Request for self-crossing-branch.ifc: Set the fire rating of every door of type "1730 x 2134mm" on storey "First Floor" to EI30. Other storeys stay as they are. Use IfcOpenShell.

First a look at what the model holds.

```python
import ifcopenshell
import ifcopenshell.util.element

model = ifcopenshell.open("self-crossing-branch.ifc")
print(model.schema)
storey = next(s for s in model.by_type("IfcBuildingStorey") if s.Name == "First Floor")
doors = [e for e in ifcopenshell.util.element.get_decomposition(storey) if e.is_a("IfcDoor")]
seen = {}
for e in doors:
    element_type = ifcopenshell.util.element.get_type(e)
    key = (element_type.Name if element_type != e and element_type else None, ifcopenshell.util.element.get_pset(e, "Pset_DoorCommon", "FireRating"))
    seen[key] = seen.get(key, 0) + 1
for (name, value), count in sorted(seen.items(), key=str):
    print(count, "x", name, "|", value)
```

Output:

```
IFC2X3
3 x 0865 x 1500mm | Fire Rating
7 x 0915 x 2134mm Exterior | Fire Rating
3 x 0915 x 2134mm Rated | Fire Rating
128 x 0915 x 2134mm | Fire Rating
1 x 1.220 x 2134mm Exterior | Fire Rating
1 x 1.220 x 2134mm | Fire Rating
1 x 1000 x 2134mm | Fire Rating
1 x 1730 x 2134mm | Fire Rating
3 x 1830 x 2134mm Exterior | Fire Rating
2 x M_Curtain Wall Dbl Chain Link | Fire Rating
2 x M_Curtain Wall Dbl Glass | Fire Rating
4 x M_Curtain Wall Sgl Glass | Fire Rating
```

```python
import ifcopenshell
import ifcopenshell.api.pset
import ifcopenshell.util.element

model = ifcopenshell.open("self-crossing-branch.ifc")

storey = next(s for s in model.by_type("IfcBuildingStorey") if s.Name == "First Floor")
doors = [e for e in ifcopenshell.util.element.get_decomposition(storey) if e.is_a("IfcDoor")]

count = 0
for e in doors:
    element_type = ifcopenshell.util.element.get_type(e)
    if element_type in (None, e) or element_type.Name != "1730 x 2134mm":
        continue
    # add_pset returns the element's existing set when there is one.
    pset = ifcopenshell.api.pset.add_pset(model, product=e, name="Pset_DoorCommon")
    ifcopenshell.api.pset.edit_pset(model, pset=pset, properties={"FireRating": "EI30"})
    count += 1

print(count, "doors updated")

model.write("self-crossing-branch_edited.ifc")
```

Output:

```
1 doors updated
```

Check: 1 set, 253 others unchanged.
